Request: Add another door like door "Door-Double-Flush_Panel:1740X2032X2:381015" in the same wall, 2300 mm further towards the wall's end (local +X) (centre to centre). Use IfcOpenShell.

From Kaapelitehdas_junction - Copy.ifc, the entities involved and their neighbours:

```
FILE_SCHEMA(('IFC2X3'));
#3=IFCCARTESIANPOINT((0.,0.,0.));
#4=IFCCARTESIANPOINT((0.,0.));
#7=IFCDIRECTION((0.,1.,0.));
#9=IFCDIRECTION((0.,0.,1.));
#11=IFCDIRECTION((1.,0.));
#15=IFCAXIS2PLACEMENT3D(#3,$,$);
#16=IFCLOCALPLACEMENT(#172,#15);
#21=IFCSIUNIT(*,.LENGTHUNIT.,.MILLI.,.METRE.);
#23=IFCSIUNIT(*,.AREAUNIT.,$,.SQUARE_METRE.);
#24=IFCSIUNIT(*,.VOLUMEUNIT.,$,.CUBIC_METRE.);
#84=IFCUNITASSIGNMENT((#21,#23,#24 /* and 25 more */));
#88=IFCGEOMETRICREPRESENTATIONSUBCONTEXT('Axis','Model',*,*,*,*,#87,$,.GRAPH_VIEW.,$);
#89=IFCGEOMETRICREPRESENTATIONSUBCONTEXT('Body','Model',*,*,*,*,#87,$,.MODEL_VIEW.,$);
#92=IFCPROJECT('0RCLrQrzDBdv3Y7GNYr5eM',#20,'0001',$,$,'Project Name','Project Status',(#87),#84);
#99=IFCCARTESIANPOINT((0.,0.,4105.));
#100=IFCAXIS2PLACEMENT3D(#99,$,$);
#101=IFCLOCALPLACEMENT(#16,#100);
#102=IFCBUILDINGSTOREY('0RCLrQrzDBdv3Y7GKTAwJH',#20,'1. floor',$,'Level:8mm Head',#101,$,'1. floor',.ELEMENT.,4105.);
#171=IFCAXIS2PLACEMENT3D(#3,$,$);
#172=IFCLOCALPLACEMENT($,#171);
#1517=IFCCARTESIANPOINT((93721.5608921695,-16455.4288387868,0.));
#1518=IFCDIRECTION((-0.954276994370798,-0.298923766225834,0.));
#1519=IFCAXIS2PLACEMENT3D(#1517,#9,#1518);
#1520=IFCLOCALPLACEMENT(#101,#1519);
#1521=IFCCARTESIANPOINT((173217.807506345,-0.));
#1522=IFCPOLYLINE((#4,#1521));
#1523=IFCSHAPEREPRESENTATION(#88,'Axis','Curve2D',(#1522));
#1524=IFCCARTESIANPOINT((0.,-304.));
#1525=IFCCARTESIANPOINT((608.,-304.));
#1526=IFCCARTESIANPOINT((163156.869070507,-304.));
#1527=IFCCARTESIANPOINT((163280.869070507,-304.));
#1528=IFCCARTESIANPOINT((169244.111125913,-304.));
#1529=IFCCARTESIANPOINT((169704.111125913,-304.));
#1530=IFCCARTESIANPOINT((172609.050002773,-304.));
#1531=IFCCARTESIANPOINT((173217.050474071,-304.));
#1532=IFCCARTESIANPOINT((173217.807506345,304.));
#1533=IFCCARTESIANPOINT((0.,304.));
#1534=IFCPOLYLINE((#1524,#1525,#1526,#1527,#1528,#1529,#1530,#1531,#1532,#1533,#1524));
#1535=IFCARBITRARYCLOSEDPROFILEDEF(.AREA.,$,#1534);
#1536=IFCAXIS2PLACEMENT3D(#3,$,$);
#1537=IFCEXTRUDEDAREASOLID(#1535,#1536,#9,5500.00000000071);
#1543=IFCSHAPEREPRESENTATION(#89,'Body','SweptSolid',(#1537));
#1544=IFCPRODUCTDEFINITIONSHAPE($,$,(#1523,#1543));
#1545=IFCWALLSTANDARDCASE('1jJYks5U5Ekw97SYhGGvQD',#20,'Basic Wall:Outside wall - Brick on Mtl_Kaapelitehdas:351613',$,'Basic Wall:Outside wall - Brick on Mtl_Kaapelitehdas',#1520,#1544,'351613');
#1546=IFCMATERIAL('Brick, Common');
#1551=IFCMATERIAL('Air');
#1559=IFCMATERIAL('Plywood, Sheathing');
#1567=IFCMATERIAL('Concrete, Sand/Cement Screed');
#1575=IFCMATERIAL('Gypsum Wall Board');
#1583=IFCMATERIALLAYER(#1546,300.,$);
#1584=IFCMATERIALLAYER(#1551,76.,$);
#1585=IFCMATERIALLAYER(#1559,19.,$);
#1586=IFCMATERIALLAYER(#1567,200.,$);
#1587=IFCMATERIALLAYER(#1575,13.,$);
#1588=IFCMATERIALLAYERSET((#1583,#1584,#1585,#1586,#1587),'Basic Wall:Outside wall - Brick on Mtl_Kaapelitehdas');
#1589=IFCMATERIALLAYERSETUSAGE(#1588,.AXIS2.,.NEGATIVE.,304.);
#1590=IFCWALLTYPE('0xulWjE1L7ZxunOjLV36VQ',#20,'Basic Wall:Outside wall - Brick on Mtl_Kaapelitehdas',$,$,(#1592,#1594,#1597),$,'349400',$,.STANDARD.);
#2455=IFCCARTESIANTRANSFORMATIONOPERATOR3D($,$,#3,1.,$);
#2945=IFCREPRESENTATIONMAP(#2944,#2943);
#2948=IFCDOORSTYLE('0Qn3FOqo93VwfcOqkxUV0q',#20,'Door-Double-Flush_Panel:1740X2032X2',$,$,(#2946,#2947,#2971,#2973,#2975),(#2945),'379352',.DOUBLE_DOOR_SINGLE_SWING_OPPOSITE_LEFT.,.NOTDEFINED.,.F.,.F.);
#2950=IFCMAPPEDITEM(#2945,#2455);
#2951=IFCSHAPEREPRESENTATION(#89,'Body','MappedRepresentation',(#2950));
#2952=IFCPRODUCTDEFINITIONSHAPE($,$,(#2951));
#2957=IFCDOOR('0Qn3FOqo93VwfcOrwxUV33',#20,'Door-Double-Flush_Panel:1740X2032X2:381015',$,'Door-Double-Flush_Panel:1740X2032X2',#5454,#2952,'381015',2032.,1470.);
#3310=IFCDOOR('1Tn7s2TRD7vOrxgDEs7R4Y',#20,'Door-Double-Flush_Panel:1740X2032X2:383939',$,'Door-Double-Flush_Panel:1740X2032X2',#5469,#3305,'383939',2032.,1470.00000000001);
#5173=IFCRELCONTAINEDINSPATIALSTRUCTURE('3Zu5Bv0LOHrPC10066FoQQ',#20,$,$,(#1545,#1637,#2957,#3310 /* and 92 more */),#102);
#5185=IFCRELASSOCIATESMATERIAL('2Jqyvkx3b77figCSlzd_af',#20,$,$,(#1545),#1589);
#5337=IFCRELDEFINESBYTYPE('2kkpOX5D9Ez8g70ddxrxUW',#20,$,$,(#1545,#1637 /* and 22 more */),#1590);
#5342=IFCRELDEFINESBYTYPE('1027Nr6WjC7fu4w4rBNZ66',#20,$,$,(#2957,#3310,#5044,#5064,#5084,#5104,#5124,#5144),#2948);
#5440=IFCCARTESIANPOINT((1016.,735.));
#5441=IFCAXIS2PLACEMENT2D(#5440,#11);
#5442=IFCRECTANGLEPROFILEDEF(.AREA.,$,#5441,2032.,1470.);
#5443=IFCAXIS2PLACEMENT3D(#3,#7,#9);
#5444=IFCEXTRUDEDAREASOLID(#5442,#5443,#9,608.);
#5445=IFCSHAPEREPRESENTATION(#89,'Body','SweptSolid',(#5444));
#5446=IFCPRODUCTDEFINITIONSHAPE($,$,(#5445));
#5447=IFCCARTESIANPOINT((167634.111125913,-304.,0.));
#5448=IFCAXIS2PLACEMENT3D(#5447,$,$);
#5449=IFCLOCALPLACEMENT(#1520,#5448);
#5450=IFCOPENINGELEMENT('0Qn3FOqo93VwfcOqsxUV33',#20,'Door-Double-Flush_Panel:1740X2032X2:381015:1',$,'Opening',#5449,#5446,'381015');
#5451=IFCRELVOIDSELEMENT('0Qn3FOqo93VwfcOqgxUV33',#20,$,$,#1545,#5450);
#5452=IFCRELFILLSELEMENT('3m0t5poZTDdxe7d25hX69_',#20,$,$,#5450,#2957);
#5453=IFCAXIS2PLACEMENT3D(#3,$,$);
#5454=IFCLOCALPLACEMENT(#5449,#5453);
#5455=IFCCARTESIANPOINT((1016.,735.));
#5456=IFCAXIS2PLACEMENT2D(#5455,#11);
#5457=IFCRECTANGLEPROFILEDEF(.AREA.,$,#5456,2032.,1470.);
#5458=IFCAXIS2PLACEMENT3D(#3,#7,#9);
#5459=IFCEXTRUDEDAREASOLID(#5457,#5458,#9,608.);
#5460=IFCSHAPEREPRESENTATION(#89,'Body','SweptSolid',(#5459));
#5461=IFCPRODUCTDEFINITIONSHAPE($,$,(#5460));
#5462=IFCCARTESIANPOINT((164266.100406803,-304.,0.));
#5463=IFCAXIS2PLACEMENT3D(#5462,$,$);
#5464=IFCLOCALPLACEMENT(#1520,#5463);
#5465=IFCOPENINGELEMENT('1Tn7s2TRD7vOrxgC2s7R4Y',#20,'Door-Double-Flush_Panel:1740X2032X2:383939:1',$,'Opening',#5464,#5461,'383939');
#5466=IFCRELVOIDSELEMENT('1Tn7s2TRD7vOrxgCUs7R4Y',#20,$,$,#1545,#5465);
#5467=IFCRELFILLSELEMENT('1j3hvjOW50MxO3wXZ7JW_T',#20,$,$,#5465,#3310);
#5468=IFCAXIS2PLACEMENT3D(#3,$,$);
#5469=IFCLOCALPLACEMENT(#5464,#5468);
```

```python
import ifcopenshell
import ifcopenshell.api.feature
import ifcopenshell.api.geometry
import ifcopenshell.api.root
import ifcopenshell.geom
import ifcopenshell.util.element
import ifcopenshell.util.placement
import ifcopenshell.util.shape
import ifcopenshell.util.unit

model = ifcopenshell.open("Kaapelitehdas_junction - Copy.ifc")
unit_scale = ifcopenshell.util.unit.calculate_unit_scale(model)
settings = ifcopenshell.geom.settings()


def volume(element):
    """Net volume in cubic metres, openings subtracted."""
    shape = ifcopenshell.geom.create_shape(settings, element)
    return ifcopenshell.util.shape.get_volume(shape.geometry)


def reuse_history(source, copy):
    """copy_class also copies each property set's owner history, people and application; keep the originals."""
    for rel in copy.IsDefinedBy:
        if rel.is_a("IfcRelDefinesByProperties") and (history := rel.RelatingPropertyDefinition.OwnerHistory):
            rel.RelatingPropertyDefinition.OwnerHistory = source.OwnerHistory
            ifcopenshell.util.element.remove_deep2(model, history)


door = model.by_guid("0Qn3FOqo93VwfcOrwxUV33")
opening = door.FillsVoids[0].RelatingOpeningElement
wall = opening.VoidsElements[0].RelatingBuildingElement
before = volume(wall)
shift = ifcopenshell.util.placement.get_local_placement(wall.ObjectPlacement)[:3, 0] * 2.3 / unit_scale

# copy_class copies the void relationship, type, container and properties, but no geometry.
new_opening = ifcopenshell.api.root.copy_class(model, product=opening)
new_opening.Representation = ifcopenshell.util.element.copy_deep(
    model, opening.Representation, exclude=["IfcGeometricRepresentationContext", "IfcRepresentationMap"]
)
new_opening.Name = "Door-Double-Flush_Panel:1740X2032X2"
new_opening.Tag = None
new_door = ifcopenshell.api.root.copy_class(model, product=door)
new_door.Representation = ifcopenshell.util.element.copy_deep(
    model, door.Representation, exclude=["IfcGeometricRepresentationContext", "IfcRepresentationMap"]
)
new_door.Name = "Door-Double-Flush_Panel:1740X2032X2"
new_door.Tag = None
reuse_history(door, new_door)
fills = ifcopenshell.api.feature.add_filling(model, opening=new_opening, element=new_door)
fills.OwnerHistory = new_door.OwnerHistory  # required in IFC2X3

for old, new in ((opening, new_opening), (door, new_door)):
    matrix = ifcopenshell.util.placement.get_local_placement(old.ObjectPlacement)
    matrix[:3, 3] += shift
    ifcopenshell.api.geometry.edit_object_placement(model, product=new, matrix=matrix, is_si=False)

after = volume(wall)

print(f"wall volume {before:.3f} -> {after:.3f} m3")

model.write("Kaapelitehdas_junction - Copy_v2.ifc")
```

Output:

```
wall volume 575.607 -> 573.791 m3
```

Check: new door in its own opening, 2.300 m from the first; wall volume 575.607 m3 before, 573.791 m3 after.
